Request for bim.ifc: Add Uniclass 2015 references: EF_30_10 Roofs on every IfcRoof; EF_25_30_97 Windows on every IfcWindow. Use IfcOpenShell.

First a look at what the model holds.

```python
import ifcopenshell

model = ifcopenshell.open("bim.ifc")
print(model.schema)
print("classifications:", [c.Name for c in model.by_type("IfcClassification")])
for ifc_class in ("IfcDoor", "IfcRoof", "IfcStair", "IfcWall", "IfcWindow"):
    print(ifc_class, len(model.by_type(ifc_class)))
```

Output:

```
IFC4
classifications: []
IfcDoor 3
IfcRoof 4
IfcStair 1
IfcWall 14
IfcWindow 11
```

```python
import ifcopenshell
import ifcopenshell.api.classification

model = ifcopenshell.open("bim.ifc")

system = ifcopenshell.api.classification.add_classification(model, classification="Uniclass 2015")

codes = {
    "IfcRoof": ("EF_30_10", "Roofs"),
    "IfcWindow": ("EF_25_30_97", "Windows"),
}
for ifc_class, (code, name) in codes.items():
    products = model.by_type(ifc_class)
    ifcopenshell.api.classification.add_reference(
        model, products=products, classification=system, identification=code, name=name
    )
    print(code, len(products))

model.write("bim_rev.ifc")
```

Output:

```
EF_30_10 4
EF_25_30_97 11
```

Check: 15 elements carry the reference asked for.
